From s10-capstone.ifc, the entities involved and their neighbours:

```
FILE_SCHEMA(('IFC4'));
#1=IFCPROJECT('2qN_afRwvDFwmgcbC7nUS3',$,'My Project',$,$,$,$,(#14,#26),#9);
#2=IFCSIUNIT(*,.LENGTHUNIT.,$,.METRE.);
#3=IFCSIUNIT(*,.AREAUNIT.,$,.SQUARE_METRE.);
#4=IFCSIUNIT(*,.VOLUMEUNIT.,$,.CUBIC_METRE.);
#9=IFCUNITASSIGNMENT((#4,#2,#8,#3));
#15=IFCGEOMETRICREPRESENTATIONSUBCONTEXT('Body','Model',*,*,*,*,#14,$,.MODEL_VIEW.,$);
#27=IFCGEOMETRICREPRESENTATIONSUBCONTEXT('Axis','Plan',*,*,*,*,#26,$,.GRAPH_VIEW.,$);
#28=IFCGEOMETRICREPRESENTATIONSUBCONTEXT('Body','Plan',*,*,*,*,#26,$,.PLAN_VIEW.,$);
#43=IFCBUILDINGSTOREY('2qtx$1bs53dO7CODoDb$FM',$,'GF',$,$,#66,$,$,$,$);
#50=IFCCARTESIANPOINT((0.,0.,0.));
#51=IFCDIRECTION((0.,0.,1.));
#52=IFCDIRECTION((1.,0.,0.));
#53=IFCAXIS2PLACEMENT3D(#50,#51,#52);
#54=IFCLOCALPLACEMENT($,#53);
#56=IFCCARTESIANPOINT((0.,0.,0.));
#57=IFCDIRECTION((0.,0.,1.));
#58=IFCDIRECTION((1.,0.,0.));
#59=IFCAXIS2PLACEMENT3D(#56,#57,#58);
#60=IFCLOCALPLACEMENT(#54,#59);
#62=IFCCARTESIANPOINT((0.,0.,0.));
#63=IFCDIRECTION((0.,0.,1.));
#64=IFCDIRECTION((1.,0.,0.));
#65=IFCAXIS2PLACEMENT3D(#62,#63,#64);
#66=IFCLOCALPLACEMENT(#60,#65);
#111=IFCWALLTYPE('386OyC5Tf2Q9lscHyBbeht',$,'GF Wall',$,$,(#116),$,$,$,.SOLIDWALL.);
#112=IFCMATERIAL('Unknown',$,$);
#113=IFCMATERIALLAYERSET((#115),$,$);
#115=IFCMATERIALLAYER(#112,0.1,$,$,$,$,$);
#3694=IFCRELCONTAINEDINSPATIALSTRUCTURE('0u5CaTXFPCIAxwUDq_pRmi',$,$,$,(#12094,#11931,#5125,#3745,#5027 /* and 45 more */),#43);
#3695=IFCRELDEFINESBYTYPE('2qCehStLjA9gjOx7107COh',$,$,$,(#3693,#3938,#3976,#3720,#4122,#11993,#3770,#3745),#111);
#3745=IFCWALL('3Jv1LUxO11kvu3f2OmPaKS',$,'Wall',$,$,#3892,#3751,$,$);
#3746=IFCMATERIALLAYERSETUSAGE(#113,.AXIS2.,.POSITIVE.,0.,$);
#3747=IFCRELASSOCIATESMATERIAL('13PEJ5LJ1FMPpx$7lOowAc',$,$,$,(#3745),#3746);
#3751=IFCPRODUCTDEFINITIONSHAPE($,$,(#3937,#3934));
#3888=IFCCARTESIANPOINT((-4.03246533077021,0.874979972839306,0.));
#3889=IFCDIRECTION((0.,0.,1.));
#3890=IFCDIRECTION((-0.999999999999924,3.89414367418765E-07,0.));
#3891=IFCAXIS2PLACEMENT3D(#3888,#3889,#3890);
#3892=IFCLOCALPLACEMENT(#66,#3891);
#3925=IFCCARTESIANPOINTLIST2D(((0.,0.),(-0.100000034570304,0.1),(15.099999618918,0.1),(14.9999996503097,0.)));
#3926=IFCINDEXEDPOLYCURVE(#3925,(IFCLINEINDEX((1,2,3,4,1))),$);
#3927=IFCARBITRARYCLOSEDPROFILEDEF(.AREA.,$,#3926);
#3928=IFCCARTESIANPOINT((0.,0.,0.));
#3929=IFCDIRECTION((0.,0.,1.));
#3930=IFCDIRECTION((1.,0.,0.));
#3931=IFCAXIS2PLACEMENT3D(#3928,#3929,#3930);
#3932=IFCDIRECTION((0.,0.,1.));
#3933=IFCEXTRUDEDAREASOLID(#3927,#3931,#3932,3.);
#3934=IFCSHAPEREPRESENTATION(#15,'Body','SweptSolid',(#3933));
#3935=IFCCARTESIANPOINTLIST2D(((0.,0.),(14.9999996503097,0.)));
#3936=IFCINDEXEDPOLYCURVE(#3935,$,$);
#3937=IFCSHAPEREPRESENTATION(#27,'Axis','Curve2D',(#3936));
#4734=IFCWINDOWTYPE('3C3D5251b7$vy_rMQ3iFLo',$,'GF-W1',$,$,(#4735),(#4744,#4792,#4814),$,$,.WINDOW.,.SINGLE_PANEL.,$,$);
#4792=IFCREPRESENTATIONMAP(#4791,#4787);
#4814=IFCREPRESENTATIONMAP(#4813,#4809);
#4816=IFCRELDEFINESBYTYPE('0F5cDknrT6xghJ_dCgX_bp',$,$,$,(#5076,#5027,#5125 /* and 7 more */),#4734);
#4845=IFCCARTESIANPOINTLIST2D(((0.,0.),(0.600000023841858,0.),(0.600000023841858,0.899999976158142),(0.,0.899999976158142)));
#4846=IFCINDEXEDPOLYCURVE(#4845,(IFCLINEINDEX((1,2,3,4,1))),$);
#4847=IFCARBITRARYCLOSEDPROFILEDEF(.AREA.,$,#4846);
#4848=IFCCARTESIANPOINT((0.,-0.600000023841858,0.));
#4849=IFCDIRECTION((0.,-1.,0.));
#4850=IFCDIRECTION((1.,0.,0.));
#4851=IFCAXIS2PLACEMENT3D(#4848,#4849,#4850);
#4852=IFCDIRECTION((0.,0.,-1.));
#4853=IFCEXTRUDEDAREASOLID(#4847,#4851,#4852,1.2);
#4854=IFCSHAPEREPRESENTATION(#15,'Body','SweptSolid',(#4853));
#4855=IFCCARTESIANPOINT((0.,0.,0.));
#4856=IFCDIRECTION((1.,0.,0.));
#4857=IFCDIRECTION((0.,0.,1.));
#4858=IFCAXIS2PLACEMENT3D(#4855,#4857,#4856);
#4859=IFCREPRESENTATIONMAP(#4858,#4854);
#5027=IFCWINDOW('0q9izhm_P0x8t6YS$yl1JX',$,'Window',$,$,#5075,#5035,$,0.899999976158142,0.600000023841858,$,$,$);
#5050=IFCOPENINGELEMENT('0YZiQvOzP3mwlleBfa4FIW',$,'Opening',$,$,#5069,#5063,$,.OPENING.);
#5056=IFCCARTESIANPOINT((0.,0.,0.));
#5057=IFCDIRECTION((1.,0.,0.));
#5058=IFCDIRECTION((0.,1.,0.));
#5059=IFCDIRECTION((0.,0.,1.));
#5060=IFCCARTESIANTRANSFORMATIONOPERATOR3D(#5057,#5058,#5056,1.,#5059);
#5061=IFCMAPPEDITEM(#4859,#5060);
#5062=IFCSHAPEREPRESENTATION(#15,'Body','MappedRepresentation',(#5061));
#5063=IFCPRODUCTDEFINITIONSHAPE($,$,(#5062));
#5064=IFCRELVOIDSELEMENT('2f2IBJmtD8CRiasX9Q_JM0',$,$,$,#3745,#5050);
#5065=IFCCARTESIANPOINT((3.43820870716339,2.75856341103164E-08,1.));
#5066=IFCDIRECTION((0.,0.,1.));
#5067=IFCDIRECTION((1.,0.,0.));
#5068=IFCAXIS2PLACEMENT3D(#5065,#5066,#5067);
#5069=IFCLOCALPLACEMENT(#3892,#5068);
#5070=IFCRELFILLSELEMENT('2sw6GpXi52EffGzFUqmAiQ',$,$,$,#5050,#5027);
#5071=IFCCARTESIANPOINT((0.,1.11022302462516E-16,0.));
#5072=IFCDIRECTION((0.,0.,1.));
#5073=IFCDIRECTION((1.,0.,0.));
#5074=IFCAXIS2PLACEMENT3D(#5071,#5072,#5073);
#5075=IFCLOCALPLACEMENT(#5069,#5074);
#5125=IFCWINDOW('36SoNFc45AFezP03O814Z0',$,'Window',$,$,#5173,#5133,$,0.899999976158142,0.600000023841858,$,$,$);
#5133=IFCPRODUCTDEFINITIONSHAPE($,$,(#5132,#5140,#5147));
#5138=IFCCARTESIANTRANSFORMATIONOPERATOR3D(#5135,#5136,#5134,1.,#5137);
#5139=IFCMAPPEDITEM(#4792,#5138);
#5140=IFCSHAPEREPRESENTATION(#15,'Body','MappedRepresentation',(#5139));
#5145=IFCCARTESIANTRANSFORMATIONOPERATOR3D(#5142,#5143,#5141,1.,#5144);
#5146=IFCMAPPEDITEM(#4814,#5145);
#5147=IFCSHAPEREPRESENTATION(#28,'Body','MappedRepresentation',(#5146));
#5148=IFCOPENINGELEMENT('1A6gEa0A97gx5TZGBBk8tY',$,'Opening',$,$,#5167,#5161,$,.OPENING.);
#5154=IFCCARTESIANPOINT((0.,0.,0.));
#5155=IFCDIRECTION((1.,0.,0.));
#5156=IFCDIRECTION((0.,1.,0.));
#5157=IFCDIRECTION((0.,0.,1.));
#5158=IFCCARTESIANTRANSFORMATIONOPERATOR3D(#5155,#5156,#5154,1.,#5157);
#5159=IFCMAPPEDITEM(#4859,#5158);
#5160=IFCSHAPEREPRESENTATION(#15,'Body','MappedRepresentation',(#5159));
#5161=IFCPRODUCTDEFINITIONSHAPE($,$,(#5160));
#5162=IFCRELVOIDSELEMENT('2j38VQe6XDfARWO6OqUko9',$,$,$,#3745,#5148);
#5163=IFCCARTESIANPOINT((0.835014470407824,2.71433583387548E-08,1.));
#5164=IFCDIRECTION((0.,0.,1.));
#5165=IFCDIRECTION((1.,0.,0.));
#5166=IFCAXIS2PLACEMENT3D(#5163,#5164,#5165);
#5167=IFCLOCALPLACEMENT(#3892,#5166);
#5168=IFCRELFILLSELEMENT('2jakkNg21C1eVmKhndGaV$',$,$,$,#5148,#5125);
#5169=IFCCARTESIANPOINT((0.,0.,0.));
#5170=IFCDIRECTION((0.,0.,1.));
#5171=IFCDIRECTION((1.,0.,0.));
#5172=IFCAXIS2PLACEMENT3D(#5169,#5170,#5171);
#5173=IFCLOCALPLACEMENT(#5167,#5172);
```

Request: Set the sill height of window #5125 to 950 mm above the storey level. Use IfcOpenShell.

```python
import numpy as np
import ifcopenshell
import ifcopenshell.api.geometry
import ifcopenshell.geom
import ifcopenshell.util.element
import ifcopenshell.util.placement
import ifcopenshell.util.shape
import ifcopenshell.util.unit

model = ifcopenshell.open("s10-capstone.ifc")
unit_scale = ifcopenshell.util.unit.calculate_unit_scale(model)

window = model.by_guid("36SoNFc45AFezP03O814Z0")
opening = window.FillsVoids[0].RelatingOpeningElement
storey = ifcopenshell.util.element.get_container(window, ifc_class="IfcBuildingStorey")
level = ifcopenshell.util.placement.get_local_placement(storey.ObjectPlacement)[2, 3]

# The opening's origin need not be at the sill, so measure its lowest point.
shape = ifcopenshell.geom.create_shape(ifcopenshell.geom.settings(), opening)
bottom = ifcopenshell.util.shape.get_shape_bottom_elevation(shape, shape.geometry) / unit_scale
dz = level + 0.95 - bottom

shift = np.array([0.0, 0.0, dz])
# The window is placed relative to its opening, so it follows when the opening moves.
matrix = ifcopenshell.util.placement.get_local_placement(opening.ObjectPlacement)
matrix[:3, 3] += shift
ifcopenshell.api.geometry.edit_object_placement(
    model, product=opening, matrix=matrix, is_si=False, should_transform_children=True
)

print(f"moved by {dz * unit_scale:+.3f} m")

model.write("s10-capstone_v2.ifc")
```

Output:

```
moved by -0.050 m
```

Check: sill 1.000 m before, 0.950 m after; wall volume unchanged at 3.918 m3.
